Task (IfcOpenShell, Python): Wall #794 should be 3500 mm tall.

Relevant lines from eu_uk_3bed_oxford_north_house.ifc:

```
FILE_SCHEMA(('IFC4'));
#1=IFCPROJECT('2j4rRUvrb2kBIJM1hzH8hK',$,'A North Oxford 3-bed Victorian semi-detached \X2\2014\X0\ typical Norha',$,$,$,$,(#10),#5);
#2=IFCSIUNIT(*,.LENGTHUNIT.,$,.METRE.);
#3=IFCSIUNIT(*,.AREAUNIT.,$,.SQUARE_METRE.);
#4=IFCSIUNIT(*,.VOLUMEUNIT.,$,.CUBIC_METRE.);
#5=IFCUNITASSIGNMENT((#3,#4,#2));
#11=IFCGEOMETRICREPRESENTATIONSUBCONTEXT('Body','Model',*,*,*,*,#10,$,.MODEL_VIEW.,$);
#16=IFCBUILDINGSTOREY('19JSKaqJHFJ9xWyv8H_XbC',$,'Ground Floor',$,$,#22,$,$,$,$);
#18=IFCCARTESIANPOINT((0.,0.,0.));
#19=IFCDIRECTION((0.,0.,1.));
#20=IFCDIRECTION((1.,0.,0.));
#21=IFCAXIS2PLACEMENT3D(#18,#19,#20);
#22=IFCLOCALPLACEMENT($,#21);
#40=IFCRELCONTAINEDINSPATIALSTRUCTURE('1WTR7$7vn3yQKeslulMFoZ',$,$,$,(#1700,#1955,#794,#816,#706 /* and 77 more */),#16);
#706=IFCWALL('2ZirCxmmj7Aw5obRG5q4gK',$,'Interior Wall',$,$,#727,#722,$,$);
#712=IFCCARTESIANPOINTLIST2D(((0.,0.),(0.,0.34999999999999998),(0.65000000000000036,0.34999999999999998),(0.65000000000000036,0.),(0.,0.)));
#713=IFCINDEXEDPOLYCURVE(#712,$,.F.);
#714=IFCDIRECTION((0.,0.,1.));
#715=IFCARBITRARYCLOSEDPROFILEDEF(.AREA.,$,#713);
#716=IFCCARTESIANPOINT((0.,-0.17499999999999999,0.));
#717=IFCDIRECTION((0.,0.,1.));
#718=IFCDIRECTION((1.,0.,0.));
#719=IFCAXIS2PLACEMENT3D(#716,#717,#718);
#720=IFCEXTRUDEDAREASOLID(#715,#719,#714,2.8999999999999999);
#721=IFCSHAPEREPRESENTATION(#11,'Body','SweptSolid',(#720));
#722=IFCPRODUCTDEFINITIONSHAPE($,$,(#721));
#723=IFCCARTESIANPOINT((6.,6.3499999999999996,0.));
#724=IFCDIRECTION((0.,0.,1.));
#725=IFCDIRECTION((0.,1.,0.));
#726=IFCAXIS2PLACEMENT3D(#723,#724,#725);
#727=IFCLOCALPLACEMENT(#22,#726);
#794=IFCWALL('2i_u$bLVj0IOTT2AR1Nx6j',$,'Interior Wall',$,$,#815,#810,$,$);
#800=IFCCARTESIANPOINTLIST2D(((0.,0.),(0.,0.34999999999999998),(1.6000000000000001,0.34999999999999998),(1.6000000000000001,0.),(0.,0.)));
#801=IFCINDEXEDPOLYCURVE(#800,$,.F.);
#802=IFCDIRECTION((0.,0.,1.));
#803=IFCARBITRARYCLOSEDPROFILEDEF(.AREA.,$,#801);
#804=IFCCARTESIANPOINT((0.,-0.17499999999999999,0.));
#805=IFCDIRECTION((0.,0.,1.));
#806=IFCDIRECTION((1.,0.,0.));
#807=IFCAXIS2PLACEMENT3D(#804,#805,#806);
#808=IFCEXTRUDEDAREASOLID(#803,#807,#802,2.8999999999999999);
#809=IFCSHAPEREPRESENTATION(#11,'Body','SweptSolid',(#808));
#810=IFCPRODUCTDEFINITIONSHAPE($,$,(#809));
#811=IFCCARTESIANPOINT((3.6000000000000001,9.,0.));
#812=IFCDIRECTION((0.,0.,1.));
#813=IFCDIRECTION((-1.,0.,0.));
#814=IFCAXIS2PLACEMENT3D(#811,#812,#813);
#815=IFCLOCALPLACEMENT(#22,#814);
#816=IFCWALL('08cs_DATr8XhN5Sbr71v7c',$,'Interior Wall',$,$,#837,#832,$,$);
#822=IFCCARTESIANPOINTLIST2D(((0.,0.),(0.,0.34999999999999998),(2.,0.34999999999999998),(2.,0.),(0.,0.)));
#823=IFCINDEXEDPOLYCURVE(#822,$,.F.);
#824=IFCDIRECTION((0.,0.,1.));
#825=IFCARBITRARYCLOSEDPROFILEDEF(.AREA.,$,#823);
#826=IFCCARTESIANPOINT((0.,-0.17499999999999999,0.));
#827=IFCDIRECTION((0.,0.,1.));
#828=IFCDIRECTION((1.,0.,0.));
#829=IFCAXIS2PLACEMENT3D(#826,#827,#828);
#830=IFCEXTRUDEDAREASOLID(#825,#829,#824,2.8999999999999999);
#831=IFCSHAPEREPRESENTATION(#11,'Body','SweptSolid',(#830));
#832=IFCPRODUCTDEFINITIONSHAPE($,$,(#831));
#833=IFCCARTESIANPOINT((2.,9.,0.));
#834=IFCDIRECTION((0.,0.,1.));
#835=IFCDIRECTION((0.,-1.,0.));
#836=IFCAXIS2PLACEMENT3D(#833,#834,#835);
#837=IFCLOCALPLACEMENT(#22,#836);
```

```python
import ifcopenshell
import ifcopenshell.geom
import ifcopenshell.util.representation
import ifcopenshell.util.shape

model = ifcopenshell.open("eu_uk_3bed_oxford_north_house.ifc")
settings = ifcopenshell.geom.settings()


def volume(element):
    """Net volume in cubic metres, openings subtracted."""
    shape = ifcopenshell.geom.create_shape(settings, element)
    return ifcopenshell.util.shape.get_volume(shape.geometry)


wall = model.by_guid("2i_u$bLVj0IOTT2AR1Nx6j")
before = volume(wall)

body = ifcopenshell.util.representation.get_representation(wall, "Model", "Body")
solid = body.Items[0]
old_height = solid.Depth
solid.Depth = 3.5
after = volume(wall)

print(f"height {old_height:g} -> {solid.Depth:g}, volume {before:.3f} -> {after:.3f} m3")

model.write("eu_uk_3bed_oxford_north_house_v2.ifc")
```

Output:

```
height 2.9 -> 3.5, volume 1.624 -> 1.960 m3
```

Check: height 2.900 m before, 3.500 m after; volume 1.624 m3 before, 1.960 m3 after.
